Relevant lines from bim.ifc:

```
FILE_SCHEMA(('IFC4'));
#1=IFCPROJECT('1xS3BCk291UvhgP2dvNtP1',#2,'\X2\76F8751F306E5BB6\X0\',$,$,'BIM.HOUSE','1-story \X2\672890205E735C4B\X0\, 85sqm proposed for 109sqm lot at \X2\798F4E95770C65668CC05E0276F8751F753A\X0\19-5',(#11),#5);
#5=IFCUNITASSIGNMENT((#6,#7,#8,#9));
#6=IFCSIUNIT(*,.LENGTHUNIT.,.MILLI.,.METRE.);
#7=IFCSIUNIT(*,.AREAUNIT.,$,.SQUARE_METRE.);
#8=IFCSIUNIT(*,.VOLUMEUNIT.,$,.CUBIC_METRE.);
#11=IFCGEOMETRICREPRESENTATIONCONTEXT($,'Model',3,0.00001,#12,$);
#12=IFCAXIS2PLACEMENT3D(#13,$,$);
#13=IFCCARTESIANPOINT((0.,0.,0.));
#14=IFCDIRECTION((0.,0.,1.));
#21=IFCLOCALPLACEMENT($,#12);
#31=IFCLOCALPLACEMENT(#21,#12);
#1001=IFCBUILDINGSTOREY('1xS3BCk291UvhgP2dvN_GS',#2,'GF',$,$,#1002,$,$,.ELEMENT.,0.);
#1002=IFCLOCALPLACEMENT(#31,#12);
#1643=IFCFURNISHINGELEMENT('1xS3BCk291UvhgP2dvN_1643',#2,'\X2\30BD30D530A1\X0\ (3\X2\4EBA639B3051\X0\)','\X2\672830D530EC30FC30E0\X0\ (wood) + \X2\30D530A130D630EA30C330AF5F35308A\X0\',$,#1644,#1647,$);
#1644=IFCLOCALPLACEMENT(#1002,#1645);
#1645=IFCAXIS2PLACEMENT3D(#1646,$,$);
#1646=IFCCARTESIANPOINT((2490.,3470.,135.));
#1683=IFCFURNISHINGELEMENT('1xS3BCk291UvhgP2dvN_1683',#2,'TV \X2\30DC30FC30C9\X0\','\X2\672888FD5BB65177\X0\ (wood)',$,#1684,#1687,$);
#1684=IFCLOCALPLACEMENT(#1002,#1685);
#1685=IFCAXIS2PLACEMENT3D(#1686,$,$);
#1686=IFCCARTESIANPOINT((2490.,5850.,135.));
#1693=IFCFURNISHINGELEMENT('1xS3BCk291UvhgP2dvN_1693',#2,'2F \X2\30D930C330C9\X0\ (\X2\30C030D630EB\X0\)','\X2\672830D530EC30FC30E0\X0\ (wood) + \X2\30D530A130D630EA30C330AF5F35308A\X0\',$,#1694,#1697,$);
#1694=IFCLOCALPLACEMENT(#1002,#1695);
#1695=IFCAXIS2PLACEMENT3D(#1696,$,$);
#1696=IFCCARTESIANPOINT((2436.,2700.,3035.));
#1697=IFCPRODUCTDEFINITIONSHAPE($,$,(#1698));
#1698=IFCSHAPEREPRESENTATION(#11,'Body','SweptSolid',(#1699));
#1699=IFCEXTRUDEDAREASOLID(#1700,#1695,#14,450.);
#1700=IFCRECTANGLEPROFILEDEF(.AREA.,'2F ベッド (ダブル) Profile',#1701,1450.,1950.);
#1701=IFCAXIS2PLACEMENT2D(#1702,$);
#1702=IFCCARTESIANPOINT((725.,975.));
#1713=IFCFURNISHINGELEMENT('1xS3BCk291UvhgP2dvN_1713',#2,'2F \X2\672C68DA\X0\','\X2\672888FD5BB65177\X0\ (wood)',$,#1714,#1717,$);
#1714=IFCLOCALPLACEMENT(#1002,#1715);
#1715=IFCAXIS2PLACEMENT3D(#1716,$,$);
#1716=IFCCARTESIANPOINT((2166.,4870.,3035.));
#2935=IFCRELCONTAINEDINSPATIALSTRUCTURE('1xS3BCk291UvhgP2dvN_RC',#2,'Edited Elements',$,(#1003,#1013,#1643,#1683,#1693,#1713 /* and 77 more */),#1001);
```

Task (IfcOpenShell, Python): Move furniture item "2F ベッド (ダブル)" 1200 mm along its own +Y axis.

```python
import ifcopenshell
import ifcopenshell.api.geometry
import ifcopenshell.util.placement
import ifcopenshell.util.unit

model = ifcopenshell.open("bim.ifc")
unit_scale = ifcopenshell.util.unit.calculate_unit_scale(model)

item = model.by_id(1693)
matrix = ifcopenshell.util.placement.get_local_placement(item.ObjectPlacement)
matrix[:3, 3] += matrix[:3, 1] * 1.2 / unit_scale
ifcopenshell.api.geometry.edit_object_placement(model, product=item, matrix=matrix, is_si=False)

print(ifcopenshell.util.placement.get_local_placement(item.ObjectPlacement).round(3) + 0.0)

model.write("bim_v2.ifc")
```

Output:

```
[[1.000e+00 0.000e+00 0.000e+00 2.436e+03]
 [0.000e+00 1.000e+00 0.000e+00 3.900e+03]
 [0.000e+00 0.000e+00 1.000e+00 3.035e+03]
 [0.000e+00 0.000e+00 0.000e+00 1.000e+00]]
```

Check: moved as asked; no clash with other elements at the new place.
